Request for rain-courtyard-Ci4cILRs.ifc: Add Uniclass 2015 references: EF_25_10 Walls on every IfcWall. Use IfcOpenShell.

First a look at what the model holds.

```python
import ifcopenshell

model = ifcopenshell.open("rain-courtyard-Ci4cILRs.ifc")
print(model.schema)
print("classifications:", [c.Name for c in model.by_type("IfcClassification")])
for ifc_class in ("IfcDoor", "IfcRoof", "IfcStair", "IfcWall", "IfcWindow"):
    print(ifc_class, len(model.by_type(ifc_class)))
```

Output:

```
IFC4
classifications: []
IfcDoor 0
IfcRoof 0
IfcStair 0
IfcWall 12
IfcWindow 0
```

```python
import ifcopenshell
import ifcopenshell.api.classification

model = ifcopenshell.open("rain-courtyard-Ci4cILRs.ifc")

system = ifcopenshell.api.classification.add_classification(model, classification="Uniclass 2015")

codes = {
    "IfcWall": ("EF_25_10", "Walls"),
}
for ifc_class, (code, name) in codes.items():
    products = model.by_type(ifc_class)
    ifcopenshell.api.classification.add_reference(
        model, products=products, classification=system, identification=code, name=name
    )
    print(code, len(products))

model.write("rain-courtyard-Ci4cILRs_edited.ifc")
```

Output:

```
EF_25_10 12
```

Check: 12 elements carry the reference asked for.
